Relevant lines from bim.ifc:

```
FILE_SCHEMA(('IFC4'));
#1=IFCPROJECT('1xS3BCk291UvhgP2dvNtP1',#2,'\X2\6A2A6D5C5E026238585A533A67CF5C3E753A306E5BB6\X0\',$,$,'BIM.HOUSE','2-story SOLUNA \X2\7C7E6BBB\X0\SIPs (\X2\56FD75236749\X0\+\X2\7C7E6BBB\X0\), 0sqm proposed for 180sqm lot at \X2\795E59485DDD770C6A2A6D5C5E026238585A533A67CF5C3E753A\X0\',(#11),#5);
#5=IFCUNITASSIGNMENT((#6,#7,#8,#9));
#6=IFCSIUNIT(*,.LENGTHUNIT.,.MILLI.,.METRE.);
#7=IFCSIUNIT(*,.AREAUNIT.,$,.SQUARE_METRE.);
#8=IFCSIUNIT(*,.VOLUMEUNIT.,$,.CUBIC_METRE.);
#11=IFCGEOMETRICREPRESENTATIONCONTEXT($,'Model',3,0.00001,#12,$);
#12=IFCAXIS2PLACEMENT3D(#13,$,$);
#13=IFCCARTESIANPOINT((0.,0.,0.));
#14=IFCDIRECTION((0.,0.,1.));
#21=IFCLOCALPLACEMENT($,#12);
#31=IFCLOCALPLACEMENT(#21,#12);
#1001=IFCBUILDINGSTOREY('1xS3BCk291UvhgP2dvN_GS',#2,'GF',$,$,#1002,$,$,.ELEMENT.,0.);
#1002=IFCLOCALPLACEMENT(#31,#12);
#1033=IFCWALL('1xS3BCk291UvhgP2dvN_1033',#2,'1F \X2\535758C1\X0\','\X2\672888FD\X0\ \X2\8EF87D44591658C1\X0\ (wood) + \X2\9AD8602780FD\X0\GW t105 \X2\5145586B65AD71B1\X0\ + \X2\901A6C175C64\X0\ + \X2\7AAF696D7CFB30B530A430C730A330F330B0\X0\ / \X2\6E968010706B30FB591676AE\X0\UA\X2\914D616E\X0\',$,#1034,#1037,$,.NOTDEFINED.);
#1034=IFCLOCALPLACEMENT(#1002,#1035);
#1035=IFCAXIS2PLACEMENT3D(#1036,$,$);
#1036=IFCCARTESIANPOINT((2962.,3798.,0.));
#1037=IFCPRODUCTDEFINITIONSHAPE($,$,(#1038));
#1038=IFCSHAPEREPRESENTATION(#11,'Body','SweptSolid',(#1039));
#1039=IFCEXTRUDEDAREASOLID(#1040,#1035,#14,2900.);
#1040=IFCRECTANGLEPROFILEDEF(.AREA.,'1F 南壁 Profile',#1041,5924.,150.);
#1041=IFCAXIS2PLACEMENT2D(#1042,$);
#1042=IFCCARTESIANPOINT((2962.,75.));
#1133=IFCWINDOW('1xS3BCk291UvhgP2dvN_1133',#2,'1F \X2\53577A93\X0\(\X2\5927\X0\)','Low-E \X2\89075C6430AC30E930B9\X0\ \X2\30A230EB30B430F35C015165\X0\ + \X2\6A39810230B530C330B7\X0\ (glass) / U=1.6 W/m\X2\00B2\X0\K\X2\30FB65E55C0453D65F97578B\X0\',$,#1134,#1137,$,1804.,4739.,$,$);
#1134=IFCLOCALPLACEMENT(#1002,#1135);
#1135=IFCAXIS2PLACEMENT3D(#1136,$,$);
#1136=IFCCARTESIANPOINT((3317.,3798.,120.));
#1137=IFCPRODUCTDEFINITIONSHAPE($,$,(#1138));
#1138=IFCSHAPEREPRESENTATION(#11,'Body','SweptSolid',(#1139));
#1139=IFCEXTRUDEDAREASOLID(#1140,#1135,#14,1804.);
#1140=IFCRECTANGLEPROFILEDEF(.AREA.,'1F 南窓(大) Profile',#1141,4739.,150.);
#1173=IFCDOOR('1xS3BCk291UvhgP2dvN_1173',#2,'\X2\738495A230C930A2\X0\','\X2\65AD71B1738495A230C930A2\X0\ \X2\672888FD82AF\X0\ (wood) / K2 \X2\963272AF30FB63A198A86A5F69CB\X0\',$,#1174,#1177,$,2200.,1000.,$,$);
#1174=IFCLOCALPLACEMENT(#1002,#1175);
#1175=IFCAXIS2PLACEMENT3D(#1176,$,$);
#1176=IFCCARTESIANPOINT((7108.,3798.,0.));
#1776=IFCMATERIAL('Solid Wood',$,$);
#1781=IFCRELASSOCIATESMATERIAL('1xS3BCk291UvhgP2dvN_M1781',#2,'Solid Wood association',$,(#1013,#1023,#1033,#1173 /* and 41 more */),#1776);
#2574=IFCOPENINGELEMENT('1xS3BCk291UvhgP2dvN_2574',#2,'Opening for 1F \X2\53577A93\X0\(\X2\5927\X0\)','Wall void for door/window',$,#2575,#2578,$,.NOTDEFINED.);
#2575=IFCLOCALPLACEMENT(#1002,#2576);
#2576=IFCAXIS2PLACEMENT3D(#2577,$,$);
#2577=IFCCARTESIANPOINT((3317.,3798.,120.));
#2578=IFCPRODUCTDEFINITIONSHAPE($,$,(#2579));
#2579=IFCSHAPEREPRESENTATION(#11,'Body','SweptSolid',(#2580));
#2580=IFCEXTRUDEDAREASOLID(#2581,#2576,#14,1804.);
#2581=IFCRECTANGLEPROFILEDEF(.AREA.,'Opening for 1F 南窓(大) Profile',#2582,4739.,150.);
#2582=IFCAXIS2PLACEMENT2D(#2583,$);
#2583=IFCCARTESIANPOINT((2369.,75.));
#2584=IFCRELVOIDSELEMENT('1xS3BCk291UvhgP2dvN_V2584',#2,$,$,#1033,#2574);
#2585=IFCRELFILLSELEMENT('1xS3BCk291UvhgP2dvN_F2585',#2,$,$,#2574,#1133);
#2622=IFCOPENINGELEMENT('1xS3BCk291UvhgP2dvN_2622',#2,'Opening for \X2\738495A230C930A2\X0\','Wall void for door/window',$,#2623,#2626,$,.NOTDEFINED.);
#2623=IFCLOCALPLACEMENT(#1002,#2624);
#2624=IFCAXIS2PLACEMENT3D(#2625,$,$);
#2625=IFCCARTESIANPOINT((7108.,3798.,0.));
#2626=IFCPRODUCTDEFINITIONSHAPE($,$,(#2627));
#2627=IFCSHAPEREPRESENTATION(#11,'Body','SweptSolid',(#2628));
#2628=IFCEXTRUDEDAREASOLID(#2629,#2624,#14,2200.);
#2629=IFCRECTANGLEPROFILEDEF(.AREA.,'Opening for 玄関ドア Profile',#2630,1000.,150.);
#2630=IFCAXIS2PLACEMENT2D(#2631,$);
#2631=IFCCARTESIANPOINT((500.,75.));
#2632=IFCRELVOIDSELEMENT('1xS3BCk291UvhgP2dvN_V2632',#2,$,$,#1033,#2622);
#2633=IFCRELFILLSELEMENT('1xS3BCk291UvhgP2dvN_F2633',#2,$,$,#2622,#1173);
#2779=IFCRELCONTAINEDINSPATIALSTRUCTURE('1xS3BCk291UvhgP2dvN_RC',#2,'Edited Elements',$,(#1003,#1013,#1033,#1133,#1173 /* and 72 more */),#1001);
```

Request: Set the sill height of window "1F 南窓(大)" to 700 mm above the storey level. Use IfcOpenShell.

```python
import numpy as np
import ifcopenshell
import ifcopenshell.api.geometry
import ifcopenshell.geom
import ifcopenshell.util.element
import ifcopenshell.util.placement
import ifcopenshell.util.shape
import ifcopenshell.util.unit

model = ifcopenshell.open("bim.ifc")
unit_scale = ifcopenshell.util.unit.calculate_unit_scale(model)

window = model.by_guid("1xS3BCk291UvhgP2dvN_1133")
opening = window.FillsVoids[0].RelatingOpeningElement
storey = ifcopenshell.util.element.get_container(window, ifc_class="IfcBuildingStorey")
level = ifcopenshell.util.placement.get_local_placement(storey.ObjectPlacement)[2, 3]

# The opening's origin need not be at the sill, so measure its lowest point.
shape = ifcopenshell.geom.create_shape(ifcopenshell.geom.settings(), opening)
bottom = ifcopenshell.util.shape.get_shape_bottom_elevation(shape, shape.geometry) / unit_scale
dz = level + 700.0 - bottom

shift = np.array([0.0, 0.0, dz])
# The window is not placed relative to its opening, so move both.
for product in (opening, window):
    matrix = ifcopenshell.util.placement.get_local_placement(product.ObjectPlacement)
    matrix[:3, 3] += shift
    ifcopenshell.api.geometry.edit_object_placement(model, product=product, matrix=matrix, is_si=False)

print(f"moved by {dz * unit_scale:+.3f} m")

model.write("bim_updated.ifc")
```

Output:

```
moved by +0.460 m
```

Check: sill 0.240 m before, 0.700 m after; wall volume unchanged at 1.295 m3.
